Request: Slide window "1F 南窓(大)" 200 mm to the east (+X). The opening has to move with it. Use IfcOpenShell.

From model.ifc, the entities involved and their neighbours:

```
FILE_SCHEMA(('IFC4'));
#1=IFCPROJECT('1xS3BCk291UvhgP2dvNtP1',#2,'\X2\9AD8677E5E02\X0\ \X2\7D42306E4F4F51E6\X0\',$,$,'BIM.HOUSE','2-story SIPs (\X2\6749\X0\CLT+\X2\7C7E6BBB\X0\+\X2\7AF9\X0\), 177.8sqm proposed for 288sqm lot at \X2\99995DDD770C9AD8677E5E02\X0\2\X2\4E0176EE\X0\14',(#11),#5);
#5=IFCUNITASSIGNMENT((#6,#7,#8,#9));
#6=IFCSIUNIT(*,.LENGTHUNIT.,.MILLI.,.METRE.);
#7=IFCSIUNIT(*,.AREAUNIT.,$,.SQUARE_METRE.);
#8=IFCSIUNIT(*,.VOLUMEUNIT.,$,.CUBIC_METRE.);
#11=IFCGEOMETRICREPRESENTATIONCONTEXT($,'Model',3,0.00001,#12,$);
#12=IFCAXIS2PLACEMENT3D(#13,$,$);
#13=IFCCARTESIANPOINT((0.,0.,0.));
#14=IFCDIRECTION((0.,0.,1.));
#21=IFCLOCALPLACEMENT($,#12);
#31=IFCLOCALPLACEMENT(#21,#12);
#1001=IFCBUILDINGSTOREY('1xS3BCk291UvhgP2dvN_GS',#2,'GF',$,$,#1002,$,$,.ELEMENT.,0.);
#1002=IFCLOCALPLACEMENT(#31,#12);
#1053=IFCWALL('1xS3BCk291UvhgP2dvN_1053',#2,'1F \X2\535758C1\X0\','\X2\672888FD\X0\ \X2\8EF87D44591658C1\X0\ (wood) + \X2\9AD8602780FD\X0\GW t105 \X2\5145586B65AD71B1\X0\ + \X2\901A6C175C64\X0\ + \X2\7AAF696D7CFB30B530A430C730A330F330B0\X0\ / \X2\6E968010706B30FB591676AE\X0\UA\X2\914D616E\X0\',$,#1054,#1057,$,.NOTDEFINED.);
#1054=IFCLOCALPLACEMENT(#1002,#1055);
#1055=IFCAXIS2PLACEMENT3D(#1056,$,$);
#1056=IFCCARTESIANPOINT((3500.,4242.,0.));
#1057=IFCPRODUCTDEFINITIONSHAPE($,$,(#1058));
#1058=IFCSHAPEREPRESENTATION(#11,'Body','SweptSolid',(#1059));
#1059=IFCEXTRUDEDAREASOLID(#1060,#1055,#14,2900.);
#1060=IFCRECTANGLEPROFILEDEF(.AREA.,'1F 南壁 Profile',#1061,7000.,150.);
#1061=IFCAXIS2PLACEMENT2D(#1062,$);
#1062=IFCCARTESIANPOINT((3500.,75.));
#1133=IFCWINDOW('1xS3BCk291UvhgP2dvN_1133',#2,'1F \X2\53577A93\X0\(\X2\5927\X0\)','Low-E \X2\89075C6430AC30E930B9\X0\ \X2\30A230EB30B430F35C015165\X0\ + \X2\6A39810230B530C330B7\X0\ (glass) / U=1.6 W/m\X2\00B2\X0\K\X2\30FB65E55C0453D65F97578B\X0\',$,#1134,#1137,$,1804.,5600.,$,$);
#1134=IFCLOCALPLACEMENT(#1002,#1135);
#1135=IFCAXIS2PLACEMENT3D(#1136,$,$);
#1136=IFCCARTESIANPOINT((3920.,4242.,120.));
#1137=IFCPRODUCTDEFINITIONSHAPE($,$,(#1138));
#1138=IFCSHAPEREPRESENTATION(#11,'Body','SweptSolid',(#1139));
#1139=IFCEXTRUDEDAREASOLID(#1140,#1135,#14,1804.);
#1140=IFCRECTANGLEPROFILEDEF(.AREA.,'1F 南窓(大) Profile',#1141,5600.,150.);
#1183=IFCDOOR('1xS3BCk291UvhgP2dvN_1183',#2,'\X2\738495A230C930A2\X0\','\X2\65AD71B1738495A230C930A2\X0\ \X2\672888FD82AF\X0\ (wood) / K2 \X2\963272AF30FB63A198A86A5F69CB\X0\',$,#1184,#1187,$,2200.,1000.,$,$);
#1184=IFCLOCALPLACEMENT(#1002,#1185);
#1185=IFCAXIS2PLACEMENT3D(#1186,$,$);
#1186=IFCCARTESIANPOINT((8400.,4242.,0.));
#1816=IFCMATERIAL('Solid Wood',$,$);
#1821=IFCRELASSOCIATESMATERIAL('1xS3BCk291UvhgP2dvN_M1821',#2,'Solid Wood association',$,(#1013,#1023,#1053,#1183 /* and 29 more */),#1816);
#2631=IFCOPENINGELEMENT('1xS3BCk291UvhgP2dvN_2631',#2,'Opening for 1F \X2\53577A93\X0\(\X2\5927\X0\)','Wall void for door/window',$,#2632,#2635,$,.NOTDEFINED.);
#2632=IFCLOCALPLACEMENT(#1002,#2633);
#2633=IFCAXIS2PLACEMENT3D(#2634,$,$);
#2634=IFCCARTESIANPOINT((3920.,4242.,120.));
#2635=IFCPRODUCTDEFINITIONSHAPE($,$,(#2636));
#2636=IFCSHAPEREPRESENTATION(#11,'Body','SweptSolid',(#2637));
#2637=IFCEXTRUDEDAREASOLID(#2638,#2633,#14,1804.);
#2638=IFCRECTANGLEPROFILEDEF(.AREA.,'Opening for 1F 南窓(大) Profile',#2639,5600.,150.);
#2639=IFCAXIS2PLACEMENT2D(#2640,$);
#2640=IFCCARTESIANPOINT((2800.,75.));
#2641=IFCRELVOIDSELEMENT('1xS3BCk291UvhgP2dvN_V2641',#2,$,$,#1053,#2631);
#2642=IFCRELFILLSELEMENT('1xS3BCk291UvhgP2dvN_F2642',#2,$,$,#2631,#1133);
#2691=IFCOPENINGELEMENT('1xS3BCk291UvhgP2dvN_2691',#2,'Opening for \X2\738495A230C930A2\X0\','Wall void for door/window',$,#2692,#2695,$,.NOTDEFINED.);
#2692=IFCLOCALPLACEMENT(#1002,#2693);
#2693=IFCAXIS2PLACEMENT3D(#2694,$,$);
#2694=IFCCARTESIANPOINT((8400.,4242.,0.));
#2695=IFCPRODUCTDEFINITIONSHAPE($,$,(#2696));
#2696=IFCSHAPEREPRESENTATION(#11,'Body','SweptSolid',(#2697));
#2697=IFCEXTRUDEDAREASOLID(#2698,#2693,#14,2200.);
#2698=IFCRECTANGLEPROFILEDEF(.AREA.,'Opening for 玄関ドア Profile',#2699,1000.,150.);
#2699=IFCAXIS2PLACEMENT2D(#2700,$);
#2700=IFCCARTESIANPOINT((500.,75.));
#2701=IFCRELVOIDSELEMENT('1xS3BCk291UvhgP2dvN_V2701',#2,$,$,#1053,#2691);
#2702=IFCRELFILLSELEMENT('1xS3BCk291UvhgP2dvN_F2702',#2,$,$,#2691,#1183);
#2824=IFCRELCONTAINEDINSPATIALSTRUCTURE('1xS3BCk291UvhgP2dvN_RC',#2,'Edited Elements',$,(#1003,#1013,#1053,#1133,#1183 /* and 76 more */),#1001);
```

```python
import ifcopenshell
import ifcopenshell.api.geometry
import ifcopenshell.util.placement
import ifcopenshell.util.unit

model = ifcopenshell.open("model.ifc")
unit_scale = ifcopenshell.util.unit.calculate_unit_scale(model)

window = model.by_guid("1xS3BCk291UvhgP2dvN_1133")
opening = window.FillsVoids[0].RelatingOpeningElement
wall = opening.VoidsElements[0].RelatingBuildingElement

wall_matrix = ifcopenshell.util.placement.get_local_placement(wall.ObjectPlacement)
shift = wall_matrix[:3, 0] * 0.2 / unit_scale
before = ifcopenshell.util.placement.get_local_placement(window.ObjectPlacement)[:3, 3].copy()

# The window is not placed relative to its opening, so move both.
for product in (opening, window):
    matrix = ifcopenshell.util.placement.get_local_placement(product.ObjectPlacement)
    matrix[:3, 3] += shift
    ifcopenshell.api.geometry.edit_object_placement(model, product=product, matrix=matrix, is_si=False)

after = ifcopenshell.util.placement.get_local_placement(window.ObjectPlacement)[:3, 3]
print("window moved by", (after - before).round(3) + 0.0)

model.write("model_rev.ifc")
```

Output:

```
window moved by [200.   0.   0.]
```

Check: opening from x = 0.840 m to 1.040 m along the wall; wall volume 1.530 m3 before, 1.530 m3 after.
